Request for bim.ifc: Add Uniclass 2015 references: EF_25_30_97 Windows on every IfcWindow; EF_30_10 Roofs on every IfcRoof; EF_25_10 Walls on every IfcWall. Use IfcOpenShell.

First a look at what the model holds.

```python
import ifcopenshell

model = ifcopenshell.open("bim.ifc")
print(model.schema)
print("classifications:", [c.Name for c in model.by_type("IfcClassification")])
for ifc_class in ("IfcDoor", "IfcRoof", "IfcStair", "IfcWall", "IfcWindow"):
    print(ifc_class, len(model.by_type(ifc_class)))
```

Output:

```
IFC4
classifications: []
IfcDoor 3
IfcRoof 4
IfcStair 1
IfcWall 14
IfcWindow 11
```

```python
import ifcopenshell
import ifcopenshell.api.classification

model = ifcopenshell.open("bim.ifc")

system = ifcopenshell.api.classification.add_classification(model, classification="Uniclass 2015")

codes = {
    "IfcWindow": ("EF_25_30_97", "Windows"),
    "IfcRoof": ("EF_30_10", "Roofs"),
    "IfcWall": ("EF_25_10", "Walls"),
}
for ifc_class, (code, name) in codes.items():
    products = model.by_type(ifc_class)
    ifcopenshell.api.classification.add_reference(
        model, products=products, classification=system, identification=code, name=name
    )
    print(code, len(products))

model.write("bim_v2.ifc")
```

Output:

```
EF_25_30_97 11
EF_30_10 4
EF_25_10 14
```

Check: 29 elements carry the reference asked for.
